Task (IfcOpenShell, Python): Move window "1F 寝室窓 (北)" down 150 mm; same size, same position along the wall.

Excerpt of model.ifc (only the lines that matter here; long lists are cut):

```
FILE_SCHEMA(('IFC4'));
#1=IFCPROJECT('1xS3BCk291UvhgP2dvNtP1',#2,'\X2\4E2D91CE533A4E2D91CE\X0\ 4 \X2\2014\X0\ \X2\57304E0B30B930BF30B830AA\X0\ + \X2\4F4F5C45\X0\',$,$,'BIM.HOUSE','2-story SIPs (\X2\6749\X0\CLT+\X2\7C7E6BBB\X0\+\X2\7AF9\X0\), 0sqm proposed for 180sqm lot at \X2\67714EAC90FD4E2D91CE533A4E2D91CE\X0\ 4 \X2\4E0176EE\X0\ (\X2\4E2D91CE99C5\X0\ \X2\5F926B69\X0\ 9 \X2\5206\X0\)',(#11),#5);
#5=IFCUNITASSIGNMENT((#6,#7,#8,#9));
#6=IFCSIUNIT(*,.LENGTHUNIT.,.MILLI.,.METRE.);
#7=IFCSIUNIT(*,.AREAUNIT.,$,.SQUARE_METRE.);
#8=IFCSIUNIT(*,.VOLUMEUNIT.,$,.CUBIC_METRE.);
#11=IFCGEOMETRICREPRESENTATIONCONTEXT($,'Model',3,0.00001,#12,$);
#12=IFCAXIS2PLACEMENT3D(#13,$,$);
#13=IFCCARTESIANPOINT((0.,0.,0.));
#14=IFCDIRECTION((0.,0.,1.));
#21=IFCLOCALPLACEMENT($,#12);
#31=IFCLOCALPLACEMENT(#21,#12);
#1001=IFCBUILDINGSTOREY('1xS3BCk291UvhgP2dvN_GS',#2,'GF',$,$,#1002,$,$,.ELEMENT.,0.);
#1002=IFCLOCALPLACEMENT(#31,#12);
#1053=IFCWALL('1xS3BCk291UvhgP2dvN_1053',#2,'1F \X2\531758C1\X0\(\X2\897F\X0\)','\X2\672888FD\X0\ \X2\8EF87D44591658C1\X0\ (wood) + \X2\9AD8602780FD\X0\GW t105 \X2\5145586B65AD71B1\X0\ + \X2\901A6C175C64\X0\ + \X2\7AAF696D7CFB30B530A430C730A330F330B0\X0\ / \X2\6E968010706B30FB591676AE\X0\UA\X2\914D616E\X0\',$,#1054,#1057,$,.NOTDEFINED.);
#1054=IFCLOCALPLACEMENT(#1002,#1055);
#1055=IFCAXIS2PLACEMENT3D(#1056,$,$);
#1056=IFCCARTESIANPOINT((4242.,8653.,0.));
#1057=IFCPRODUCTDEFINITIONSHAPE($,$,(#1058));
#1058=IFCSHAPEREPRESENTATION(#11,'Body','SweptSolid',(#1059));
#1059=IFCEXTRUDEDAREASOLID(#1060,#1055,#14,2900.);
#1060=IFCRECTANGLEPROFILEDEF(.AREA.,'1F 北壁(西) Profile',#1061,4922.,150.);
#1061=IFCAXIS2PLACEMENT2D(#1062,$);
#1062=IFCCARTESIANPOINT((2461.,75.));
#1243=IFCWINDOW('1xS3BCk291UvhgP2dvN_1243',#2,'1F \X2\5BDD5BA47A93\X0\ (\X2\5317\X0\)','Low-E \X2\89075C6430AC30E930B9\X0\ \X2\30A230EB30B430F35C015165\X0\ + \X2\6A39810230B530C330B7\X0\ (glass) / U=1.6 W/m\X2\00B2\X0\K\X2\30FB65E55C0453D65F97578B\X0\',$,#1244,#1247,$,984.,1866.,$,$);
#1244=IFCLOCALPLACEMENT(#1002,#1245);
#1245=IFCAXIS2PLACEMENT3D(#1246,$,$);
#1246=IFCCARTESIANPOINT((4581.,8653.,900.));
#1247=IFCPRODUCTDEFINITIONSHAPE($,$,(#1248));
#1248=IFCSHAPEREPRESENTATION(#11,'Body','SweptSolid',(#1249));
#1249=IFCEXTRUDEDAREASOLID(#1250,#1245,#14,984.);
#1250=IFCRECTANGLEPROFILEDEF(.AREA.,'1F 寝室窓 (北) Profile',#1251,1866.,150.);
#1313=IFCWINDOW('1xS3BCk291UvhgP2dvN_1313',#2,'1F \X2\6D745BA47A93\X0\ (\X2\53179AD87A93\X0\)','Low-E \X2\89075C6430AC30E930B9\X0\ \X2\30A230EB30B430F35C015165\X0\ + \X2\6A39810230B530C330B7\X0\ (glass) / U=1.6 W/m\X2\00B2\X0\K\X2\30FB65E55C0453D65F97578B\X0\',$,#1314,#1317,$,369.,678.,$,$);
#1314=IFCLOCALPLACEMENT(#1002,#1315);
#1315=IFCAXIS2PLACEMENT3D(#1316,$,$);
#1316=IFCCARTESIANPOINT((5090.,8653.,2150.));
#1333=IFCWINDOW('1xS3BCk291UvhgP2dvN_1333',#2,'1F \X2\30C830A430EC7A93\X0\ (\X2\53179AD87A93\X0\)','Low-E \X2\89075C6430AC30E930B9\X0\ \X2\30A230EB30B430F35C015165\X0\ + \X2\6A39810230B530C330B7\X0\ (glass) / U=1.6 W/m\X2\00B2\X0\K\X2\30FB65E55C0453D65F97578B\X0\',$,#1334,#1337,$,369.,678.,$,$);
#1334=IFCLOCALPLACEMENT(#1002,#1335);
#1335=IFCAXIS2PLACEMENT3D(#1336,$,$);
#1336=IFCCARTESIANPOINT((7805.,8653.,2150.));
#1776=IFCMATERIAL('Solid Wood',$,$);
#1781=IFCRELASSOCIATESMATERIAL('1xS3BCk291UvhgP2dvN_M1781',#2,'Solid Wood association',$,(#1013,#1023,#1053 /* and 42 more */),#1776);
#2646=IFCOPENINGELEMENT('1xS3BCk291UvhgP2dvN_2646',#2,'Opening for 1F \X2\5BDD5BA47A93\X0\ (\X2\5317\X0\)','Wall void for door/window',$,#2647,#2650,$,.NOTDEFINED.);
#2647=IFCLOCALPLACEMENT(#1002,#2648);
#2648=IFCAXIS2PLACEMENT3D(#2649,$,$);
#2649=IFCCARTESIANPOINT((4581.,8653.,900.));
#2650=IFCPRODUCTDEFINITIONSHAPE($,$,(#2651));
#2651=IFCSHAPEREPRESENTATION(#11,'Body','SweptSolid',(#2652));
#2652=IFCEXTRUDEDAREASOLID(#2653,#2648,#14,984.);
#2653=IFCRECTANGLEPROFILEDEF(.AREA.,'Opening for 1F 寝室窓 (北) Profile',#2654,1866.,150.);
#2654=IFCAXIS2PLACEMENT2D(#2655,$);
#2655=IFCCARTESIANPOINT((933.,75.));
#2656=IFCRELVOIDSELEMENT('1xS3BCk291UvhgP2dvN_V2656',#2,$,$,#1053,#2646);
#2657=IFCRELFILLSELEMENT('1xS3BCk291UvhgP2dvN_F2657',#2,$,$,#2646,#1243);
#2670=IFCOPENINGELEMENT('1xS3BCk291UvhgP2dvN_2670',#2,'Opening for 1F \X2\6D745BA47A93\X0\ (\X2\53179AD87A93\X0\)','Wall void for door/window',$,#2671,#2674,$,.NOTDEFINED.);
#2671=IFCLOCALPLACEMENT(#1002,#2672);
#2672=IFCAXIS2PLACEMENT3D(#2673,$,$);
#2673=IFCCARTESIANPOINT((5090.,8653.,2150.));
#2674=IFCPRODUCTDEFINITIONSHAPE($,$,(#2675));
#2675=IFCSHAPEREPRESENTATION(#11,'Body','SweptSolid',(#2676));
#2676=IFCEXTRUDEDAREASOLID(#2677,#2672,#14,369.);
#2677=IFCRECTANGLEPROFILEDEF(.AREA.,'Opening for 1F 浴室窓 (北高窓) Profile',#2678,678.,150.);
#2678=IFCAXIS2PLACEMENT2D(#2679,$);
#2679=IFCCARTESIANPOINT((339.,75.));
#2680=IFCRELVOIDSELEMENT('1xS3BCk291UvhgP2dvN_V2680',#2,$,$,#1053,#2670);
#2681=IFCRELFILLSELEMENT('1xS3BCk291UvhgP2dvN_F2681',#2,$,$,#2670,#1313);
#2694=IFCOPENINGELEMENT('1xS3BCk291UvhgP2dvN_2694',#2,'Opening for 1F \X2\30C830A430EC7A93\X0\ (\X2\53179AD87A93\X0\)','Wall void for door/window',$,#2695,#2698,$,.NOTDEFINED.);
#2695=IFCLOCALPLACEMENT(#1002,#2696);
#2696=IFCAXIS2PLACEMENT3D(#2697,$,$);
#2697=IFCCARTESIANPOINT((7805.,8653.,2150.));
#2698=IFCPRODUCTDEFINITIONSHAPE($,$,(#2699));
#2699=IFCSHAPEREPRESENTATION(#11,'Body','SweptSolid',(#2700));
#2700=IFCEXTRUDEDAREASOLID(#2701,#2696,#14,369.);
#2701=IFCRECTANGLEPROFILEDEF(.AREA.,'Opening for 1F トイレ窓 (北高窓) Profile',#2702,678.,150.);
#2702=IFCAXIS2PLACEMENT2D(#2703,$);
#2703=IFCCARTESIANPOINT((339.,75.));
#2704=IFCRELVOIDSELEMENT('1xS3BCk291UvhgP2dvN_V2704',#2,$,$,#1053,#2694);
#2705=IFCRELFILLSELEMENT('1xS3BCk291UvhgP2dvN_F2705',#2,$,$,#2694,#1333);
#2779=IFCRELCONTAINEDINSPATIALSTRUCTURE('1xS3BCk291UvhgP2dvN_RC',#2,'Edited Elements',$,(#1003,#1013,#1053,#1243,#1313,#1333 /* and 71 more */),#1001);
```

```python
import numpy as np
import ifcopenshell
import ifcopenshell.api.geometry
import ifcopenshell.util.placement
import ifcopenshell.util.unit

model = ifcopenshell.open("model.ifc")
unit_scale = ifcopenshell.util.unit.calculate_unit_scale(model)

window = model.by_guid("1xS3BCk291UvhgP2dvN_1243")
opening = window.FillsVoids[0].RelatingOpeningElement
dz = -0.15 / unit_scale

shift = np.array([0.0, 0.0, dz])
# The window is not placed relative to its opening, so move both.
for product in (opening, window):
    matrix = ifcopenshell.util.placement.get_local_placement(product.ObjectPlacement)
    matrix[:3, 3] += shift
    ifcopenshell.api.geometry.edit_object_placement(model, product=product, matrix=matrix, is_si=False)

print(f"moved by {dz * unit_scale:+.3f} m")

model.write("model_v2.ifc")
```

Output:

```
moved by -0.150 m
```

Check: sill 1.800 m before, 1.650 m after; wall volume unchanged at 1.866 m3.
